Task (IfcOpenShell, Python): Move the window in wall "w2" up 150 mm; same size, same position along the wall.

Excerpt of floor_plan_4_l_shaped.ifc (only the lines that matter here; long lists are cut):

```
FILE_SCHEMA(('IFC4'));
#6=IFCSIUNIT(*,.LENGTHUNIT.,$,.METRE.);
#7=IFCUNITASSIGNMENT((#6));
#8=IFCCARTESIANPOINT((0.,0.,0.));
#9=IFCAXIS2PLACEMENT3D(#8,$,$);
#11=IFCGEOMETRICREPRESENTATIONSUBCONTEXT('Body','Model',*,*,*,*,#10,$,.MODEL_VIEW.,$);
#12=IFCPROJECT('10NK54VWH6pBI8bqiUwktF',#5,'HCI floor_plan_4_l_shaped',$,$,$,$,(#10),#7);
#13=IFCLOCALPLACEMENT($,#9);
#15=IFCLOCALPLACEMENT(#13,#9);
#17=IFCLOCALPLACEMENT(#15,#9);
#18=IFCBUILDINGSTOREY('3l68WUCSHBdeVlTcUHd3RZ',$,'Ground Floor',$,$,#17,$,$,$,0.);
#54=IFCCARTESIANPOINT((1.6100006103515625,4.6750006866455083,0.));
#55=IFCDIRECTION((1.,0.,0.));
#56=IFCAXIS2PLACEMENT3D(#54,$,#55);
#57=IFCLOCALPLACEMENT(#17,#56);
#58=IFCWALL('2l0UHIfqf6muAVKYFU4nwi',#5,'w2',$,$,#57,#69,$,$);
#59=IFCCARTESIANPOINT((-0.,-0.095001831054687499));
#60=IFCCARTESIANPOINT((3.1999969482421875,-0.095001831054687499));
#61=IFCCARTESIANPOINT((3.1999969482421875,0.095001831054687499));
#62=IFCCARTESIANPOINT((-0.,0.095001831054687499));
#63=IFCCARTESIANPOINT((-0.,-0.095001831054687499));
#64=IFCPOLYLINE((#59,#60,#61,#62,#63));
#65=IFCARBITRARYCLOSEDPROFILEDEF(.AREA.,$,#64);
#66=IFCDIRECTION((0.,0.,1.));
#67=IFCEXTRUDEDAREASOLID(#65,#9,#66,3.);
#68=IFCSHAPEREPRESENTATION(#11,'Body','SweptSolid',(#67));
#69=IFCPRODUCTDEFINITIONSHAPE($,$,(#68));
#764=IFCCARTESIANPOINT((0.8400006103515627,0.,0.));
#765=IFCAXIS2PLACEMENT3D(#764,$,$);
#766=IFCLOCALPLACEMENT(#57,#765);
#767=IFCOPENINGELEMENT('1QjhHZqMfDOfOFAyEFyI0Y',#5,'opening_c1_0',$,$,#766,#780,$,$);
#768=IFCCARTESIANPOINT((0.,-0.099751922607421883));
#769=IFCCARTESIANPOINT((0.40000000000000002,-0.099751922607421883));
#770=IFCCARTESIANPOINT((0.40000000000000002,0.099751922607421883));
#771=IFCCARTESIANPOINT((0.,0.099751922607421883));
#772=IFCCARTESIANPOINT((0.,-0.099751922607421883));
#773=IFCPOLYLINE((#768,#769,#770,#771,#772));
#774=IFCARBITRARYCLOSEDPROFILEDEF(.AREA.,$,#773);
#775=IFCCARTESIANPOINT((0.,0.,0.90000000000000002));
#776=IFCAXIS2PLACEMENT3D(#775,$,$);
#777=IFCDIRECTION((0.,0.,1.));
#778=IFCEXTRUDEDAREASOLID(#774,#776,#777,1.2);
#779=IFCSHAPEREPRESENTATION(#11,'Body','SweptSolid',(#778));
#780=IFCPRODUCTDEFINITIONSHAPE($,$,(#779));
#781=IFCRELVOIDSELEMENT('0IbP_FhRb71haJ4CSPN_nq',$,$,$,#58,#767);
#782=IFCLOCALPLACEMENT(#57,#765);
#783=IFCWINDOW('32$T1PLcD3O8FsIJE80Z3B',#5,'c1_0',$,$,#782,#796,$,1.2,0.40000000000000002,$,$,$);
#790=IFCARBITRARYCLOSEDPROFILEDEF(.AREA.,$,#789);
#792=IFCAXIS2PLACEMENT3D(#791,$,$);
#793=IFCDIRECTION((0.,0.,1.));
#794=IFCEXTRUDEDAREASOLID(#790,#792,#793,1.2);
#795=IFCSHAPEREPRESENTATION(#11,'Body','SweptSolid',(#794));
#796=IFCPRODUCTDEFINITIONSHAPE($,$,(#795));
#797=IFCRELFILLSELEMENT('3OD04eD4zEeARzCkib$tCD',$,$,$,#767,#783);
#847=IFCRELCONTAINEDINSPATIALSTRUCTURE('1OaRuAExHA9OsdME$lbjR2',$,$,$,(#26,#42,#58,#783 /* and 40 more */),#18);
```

```python
import numpy as np
import ifcopenshell
import ifcopenshell.api.geometry
import ifcopenshell.util.placement
import ifcopenshell.util.unit

model = ifcopenshell.open("floor_plan_4_l_shaped.ifc")
unit_scale = ifcopenshell.util.unit.calculate_unit_scale(model)

window = model.by_guid("32$T1PLcD3O8FsIJE80Z3B")
opening = window.FillsVoids[0].RelatingOpeningElement
dz = 0.15 / unit_scale

shift = np.array([0.0, 0.0, dz])
# The window is not placed relative to its opening, so move both.
for product in (opening, window):
    matrix = ifcopenshell.util.placement.get_local_placement(product.ObjectPlacement)
    matrix[:3, 3] += shift
    ifcopenshell.api.geometry.edit_object_placement(model, product=product, matrix=matrix, is_si=False)

print(f"moved by {dz * unit_scale:+.3f} m")

model.write("floor_plan_4_l_shaped_v2.ifc")
```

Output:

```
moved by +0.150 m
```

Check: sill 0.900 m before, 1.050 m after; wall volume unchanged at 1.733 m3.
